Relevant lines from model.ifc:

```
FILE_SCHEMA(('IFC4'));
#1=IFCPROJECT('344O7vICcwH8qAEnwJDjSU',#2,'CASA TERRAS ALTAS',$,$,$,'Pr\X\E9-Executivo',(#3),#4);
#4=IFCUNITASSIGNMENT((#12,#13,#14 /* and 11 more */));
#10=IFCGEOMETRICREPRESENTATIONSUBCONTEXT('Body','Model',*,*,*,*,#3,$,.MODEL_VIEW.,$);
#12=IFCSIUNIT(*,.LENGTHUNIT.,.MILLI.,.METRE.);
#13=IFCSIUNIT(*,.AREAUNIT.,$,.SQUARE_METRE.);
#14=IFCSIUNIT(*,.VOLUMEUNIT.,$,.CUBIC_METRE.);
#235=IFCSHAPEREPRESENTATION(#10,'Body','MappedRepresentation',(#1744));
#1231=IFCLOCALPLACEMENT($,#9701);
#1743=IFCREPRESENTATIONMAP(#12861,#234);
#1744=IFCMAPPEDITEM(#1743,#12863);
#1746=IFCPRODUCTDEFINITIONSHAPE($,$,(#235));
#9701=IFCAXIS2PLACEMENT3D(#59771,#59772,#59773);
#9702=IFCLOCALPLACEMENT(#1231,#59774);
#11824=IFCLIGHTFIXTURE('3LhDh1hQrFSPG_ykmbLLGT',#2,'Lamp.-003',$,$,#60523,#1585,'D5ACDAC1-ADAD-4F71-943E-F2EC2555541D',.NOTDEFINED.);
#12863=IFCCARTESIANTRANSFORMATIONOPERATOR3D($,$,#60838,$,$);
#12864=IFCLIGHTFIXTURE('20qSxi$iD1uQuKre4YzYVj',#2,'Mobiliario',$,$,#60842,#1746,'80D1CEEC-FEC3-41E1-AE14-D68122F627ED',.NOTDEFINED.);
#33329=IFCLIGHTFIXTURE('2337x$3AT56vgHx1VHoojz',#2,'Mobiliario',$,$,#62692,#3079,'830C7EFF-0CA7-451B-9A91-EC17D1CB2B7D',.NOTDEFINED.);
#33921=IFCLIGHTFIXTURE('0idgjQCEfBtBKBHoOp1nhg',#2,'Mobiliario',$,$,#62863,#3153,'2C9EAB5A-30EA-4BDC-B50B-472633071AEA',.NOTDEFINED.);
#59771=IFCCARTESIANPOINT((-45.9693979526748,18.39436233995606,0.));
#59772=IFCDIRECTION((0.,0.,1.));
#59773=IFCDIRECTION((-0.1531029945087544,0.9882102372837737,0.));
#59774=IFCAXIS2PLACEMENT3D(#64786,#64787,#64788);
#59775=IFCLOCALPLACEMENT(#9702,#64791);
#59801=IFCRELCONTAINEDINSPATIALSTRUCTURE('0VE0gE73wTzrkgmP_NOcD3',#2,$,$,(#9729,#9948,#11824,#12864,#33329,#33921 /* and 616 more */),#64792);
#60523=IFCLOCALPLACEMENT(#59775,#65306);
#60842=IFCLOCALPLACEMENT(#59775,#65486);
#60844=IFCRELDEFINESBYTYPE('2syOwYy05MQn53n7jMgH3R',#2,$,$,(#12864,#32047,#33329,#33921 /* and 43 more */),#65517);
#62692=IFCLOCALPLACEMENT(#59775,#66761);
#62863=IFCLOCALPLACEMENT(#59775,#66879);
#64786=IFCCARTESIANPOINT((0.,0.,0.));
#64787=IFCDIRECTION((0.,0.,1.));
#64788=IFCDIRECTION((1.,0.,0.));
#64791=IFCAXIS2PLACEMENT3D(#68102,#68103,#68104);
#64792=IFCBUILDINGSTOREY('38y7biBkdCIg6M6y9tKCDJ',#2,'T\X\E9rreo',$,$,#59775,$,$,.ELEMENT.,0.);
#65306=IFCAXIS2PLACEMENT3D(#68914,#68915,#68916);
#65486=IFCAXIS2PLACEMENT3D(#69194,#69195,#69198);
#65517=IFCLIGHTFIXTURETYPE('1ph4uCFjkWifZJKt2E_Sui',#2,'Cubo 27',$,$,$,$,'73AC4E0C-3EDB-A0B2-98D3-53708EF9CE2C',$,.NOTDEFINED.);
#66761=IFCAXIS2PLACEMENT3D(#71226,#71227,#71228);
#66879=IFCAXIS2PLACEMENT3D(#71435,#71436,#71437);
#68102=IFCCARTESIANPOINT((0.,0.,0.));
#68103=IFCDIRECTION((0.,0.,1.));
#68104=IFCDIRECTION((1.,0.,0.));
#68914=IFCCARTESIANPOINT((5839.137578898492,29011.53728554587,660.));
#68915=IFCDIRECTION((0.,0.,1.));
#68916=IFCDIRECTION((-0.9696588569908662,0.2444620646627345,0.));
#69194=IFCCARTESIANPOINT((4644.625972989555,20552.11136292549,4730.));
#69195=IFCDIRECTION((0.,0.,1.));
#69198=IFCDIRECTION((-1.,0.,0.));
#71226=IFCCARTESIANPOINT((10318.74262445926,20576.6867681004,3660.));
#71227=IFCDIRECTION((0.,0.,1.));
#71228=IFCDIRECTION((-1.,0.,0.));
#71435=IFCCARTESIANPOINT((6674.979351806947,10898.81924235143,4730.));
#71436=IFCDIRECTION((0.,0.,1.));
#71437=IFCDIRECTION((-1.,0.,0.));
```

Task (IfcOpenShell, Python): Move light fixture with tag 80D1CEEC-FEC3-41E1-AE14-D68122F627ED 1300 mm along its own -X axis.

```python
import ifcopenshell
import ifcopenshell.api.geometry
import ifcopenshell.util.placement
import ifcopenshell.util.unit

model = ifcopenshell.open("model.ifc")
unit_scale = ifcopenshell.util.unit.calculate_unit_scale(model)

item = model.by_guid("20qSxi$iD1uQuKre4YzYVj")
matrix = ifcopenshell.util.placement.get_local_placement(item.ObjectPlacement)
matrix[:3, 3] -= matrix[:3, 0] * 1.3 / unit_scale
ifcopenshell.api.geometry.edit_object_placement(model, product=item, matrix=matrix, is_si=False)

print(ifcopenshell.util.placement.get_local_placement(item.ObjectPlacement).round(3) + 0.0)

model.write("model_updated.ifc")
```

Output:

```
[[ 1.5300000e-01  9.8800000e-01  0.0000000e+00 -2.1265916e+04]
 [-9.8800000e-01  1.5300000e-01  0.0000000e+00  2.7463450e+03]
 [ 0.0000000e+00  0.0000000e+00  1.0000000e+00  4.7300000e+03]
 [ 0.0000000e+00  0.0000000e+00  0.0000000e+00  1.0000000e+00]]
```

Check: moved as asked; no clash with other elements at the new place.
